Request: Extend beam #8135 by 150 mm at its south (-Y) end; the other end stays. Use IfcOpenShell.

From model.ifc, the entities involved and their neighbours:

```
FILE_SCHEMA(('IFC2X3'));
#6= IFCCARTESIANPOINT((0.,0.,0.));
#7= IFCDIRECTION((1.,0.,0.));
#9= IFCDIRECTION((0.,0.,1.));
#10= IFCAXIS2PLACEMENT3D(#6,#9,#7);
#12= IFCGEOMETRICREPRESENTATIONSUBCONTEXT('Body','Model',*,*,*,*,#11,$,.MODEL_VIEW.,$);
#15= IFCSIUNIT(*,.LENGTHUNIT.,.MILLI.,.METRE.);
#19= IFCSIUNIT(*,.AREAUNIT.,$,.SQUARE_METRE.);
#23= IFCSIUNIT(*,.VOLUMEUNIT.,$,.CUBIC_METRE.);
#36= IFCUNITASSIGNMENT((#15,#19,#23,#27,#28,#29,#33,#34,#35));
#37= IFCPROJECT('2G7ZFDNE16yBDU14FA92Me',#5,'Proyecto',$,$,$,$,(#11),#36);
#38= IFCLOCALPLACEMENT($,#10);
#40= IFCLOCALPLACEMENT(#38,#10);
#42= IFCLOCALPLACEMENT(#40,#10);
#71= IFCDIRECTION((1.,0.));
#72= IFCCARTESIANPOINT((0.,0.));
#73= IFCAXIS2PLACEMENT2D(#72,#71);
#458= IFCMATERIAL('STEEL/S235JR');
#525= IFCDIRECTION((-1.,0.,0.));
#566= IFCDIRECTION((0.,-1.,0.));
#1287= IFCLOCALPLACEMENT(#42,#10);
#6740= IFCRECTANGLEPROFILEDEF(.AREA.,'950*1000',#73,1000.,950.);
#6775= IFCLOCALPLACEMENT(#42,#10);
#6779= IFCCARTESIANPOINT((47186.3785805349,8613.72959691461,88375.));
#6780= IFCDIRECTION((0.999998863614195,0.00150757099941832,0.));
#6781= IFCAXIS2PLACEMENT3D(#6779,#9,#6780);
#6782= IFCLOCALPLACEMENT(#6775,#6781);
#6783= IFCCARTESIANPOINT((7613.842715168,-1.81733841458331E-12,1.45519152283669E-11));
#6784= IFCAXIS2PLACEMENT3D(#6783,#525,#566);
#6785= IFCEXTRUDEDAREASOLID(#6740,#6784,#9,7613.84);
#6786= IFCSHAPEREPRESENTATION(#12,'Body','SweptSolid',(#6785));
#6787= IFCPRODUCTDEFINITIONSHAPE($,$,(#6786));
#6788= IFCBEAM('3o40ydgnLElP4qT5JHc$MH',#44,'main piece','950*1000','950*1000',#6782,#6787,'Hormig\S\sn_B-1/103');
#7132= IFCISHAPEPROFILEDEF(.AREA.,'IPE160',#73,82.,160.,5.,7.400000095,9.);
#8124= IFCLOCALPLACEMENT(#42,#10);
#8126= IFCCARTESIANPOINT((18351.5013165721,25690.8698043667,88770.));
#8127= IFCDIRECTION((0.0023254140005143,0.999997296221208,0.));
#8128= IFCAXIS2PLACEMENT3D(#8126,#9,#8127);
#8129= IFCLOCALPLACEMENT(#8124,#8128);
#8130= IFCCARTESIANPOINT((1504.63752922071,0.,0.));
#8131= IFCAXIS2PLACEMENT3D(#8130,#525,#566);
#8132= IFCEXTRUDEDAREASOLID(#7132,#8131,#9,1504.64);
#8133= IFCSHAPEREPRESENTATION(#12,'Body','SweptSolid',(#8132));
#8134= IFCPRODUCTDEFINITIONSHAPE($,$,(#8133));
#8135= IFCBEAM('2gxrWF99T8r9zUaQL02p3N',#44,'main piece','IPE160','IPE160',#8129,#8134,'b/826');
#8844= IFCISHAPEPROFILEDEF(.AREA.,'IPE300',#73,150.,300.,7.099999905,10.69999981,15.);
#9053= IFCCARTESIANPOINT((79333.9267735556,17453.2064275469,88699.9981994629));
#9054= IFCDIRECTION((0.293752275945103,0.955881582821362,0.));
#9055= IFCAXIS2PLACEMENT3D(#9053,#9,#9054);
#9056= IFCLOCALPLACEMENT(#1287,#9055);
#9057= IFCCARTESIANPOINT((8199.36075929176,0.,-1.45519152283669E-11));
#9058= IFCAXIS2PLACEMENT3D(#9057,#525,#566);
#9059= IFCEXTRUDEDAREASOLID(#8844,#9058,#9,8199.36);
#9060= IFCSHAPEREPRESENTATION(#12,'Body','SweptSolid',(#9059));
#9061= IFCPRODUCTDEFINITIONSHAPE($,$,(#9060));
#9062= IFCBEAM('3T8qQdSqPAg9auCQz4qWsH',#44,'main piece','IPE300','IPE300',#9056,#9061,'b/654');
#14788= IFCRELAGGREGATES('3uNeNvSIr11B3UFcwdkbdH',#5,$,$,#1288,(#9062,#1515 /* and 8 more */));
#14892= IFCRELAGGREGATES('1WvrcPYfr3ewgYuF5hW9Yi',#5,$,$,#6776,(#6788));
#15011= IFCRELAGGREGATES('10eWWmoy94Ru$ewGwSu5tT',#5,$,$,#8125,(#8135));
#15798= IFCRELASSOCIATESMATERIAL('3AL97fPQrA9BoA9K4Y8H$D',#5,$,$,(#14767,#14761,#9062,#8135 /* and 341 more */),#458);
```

```python
import ifcopenshell
import ifcopenshell.util.representation

model = ifcopenshell.open("model.ifc")

member = model.by_id(8135)
change = 150.0

# The extrusion runs towards the end named, so only its depth changes.
body = ifcopenshell.util.representation.get_representation(member, "Model", "Body")
solid = body.Items[0]
old_length = solid.Depth
solid.Depth += change

print(f"length {old_length:g} -> {solid.Depth:g}")

model.write("model_v2.ifc")
```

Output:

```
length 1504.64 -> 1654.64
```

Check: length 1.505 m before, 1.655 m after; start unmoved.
